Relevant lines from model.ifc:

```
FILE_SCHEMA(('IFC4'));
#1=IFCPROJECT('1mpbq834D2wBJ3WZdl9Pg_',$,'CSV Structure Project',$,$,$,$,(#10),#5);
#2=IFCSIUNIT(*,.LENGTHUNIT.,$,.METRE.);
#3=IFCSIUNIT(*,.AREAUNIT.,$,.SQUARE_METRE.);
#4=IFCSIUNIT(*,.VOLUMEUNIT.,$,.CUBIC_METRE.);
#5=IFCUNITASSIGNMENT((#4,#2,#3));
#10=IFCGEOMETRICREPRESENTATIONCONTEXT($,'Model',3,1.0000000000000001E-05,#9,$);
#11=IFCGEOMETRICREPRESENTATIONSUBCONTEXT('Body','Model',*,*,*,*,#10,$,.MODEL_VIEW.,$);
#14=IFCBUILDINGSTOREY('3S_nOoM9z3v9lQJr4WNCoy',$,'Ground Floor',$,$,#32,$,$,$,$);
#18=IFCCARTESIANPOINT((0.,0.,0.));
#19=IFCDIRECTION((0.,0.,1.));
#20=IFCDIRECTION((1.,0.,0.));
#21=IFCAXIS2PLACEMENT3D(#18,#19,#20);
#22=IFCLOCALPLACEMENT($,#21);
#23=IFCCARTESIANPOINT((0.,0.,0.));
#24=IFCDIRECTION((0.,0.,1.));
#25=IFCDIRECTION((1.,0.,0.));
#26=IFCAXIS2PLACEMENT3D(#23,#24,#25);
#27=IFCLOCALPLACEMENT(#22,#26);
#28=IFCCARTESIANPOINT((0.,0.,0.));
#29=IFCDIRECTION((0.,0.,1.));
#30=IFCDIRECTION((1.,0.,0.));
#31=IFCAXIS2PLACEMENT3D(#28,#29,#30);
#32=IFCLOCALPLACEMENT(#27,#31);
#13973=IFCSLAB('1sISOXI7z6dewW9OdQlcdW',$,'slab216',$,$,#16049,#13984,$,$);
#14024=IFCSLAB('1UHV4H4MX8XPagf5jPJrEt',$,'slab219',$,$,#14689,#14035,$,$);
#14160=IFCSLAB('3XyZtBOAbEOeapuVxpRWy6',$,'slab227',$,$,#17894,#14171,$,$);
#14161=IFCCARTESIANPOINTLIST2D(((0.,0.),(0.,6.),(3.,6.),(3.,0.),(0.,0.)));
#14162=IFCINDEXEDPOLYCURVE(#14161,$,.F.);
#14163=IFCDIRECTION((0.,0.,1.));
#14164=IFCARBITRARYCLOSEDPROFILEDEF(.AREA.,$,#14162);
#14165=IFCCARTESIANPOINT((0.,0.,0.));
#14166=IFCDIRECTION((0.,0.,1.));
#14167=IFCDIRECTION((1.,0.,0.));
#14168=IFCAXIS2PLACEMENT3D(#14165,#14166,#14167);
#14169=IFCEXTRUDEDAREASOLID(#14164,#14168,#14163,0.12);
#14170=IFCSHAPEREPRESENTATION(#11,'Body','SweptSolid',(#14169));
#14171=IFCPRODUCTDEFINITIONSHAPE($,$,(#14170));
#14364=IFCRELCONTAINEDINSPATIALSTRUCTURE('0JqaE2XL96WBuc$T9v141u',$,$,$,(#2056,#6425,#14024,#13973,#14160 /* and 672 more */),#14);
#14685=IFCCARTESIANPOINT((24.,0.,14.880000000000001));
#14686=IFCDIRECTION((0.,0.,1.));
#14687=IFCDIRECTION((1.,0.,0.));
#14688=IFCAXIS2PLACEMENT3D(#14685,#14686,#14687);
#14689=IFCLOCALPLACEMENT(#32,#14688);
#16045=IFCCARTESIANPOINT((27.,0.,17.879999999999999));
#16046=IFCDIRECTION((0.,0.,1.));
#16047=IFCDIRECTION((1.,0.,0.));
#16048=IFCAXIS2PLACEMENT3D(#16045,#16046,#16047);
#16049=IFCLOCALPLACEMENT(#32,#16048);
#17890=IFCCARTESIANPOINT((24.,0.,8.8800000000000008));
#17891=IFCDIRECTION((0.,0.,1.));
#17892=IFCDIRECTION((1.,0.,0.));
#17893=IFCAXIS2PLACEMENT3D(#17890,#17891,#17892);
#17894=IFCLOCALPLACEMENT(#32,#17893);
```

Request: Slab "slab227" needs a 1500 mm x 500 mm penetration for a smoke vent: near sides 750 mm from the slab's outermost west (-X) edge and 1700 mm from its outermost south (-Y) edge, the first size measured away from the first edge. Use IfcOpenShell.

```python
import numpy as np
import ifcopenshell
import ifcopenshell.api.feature
import ifcopenshell.api.geometry
import ifcopenshell.api.root
import ifcopenshell.geom
import ifcopenshell.util.placement
import ifcopenshell.util.representation
import ifcopenshell.util.shape
import ifcopenshell.util.unit

model = ifcopenshell.open("model.ifc")
unit_scale = ifcopenshell.util.unit.calculate_unit_scale(model)
settings = ifcopenshell.geom.settings()


def volume(element):
    """Net volume in cubic metres, openings subtracted."""
    shape = ifcopenshell.geom.create_shape(settings, element)
    return ifcopenshell.util.shape.get_volume(shape.geometry)


slab = model.by_guid("3XyZtBOAbEOeapuVxpRWy6")
before = volume(slab)

# Extent in the slab's own axes, in metres. The edges named are its -X and -Y sides.
slab_shape = ifcopenshell.geom.create_shape(settings, slab)
vertices = ifcopenshell.util.shape.get_vertices(slab_shape.geometry)
x_min, y_min, bottom = vertices.min(axis=0)
top = vertices[:, 2].max()

opening = ifcopenshell.api.root.create_entity(model, ifc_class="IfcOpeningElement", name="Smoke vent opening", predefined_type="OPENING")
context = ifcopenshell.util.representation.get_context(model, "Model", "Body", "MODEL_VIEW")
width, depth = 1.5, 0.5
outline = [(0.0, 0.0), (width, 0.0), (width, depth), (0.0, depth), (0.0, 0.0)]
# Overshoot both faces by 50 mm so the cut is clean.
shape = ifcopenshell.api.geometry.add_slab_representation(
    model, context=context, depth=top - bottom + 0.1, polyline=outline
)
ifcopenshell.api.geometry.assign_representation(model, product=opening, representation=shape)

matrix = ifcopenshell.util.placement.get_local_placement(slab.ObjectPlacement)
matrix[:, 3] = matrix @ np.append(np.array([x_min + 0.75, y_min + 1.7, bottom - 0.05]) / unit_scale, 1.0)
ifcopenshell.api.geometry.edit_object_placement(model, product=opening, matrix=matrix, is_si=False)
ifcopenshell.api.feature.add_feature(model, feature=opening, element=slab)

after = volume(slab)

print(f"slab volume {before:.3f} -> {after:.3f} m3")

model.write("model_updated.ifc")
```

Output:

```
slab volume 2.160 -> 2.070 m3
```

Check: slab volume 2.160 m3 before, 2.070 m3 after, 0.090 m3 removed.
